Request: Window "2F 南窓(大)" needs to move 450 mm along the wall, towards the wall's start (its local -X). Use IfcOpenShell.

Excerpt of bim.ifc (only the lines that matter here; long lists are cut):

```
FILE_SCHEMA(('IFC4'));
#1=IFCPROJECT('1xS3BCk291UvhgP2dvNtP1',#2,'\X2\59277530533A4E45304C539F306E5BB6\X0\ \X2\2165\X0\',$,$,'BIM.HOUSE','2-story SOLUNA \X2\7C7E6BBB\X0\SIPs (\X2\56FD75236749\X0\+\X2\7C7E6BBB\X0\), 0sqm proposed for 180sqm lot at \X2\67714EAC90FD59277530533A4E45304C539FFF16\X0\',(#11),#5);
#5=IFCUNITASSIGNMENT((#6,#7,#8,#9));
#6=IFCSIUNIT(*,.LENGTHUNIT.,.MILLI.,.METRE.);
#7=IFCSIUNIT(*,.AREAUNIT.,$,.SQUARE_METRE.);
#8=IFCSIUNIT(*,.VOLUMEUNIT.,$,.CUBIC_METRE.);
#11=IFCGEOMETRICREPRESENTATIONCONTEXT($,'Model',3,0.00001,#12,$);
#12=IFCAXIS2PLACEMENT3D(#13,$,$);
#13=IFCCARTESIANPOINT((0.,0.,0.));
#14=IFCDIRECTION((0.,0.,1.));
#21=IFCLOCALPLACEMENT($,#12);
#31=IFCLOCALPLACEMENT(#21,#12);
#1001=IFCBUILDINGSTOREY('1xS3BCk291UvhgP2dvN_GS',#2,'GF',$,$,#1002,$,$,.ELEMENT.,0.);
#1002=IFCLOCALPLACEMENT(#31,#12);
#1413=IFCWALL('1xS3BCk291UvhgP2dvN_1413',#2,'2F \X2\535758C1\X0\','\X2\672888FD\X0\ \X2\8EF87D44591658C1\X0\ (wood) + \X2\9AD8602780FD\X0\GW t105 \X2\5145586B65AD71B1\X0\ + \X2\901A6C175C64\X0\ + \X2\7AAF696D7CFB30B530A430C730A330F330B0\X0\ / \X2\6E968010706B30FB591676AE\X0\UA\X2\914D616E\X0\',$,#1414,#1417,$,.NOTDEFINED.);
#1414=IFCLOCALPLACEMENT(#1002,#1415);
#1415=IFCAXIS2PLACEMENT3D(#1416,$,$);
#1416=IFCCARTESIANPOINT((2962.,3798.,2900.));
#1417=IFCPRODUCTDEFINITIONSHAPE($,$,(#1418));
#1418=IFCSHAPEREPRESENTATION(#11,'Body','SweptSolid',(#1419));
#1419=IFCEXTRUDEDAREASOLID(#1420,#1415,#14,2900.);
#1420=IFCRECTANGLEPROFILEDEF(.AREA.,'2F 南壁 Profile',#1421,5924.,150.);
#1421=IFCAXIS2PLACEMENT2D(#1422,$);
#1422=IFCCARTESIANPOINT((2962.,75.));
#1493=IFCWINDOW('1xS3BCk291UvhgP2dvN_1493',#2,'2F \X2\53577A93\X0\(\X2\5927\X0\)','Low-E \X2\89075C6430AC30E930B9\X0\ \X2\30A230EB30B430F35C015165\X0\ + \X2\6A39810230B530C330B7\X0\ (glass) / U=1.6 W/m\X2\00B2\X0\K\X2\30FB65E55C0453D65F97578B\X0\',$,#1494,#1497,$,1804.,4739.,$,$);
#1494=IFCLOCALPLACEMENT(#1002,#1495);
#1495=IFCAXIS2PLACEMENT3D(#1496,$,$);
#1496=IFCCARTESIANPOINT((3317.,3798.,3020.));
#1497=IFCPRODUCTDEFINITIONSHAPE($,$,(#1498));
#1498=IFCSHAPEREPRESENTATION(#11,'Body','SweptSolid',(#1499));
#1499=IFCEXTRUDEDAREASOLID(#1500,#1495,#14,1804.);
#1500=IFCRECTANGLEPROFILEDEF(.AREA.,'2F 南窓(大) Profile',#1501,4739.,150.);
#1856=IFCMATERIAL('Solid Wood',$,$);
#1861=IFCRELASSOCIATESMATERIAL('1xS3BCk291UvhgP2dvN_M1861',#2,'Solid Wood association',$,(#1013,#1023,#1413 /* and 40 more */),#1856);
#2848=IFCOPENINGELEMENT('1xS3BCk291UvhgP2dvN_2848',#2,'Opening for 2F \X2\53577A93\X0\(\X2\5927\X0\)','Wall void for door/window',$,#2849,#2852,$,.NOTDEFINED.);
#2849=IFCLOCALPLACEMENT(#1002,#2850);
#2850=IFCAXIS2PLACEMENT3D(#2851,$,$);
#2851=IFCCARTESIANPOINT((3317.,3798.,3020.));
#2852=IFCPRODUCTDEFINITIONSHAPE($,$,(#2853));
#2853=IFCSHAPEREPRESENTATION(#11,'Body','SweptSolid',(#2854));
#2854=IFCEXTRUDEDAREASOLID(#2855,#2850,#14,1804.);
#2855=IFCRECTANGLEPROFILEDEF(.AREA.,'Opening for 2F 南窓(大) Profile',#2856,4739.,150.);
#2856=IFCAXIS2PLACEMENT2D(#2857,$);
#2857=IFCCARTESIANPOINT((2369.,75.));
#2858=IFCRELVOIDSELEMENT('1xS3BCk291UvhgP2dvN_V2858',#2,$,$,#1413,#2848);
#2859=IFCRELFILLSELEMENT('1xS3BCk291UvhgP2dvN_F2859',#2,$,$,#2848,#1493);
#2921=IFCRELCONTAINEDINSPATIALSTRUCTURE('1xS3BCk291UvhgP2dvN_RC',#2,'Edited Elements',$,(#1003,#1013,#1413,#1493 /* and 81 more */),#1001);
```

```python
import ifcopenshell
import ifcopenshell.api.geometry
import ifcopenshell.util.placement
import ifcopenshell.util.unit

model = ifcopenshell.open("bim.ifc")
unit_scale = ifcopenshell.util.unit.calculate_unit_scale(model)

window = model.by_id(1493)
opening = window.FillsVoids[0].RelatingOpeningElement
wall = opening.VoidsElements[0].RelatingBuildingElement

wall_matrix = ifcopenshell.util.placement.get_local_placement(wall.ObjectPlacement)
shift = wall_matrix[:3, 0] * -0.45 / unit_scale
before = ifcopenshell.util.placement.get_local_placement(window.ObjectPlacement)[:3, 3].copy()

# The window is not placed relative to its opening, so move both.
for product in (opening, window):
    matrix = ifcopenshell.util.placement.get_local_placement(product.ObjectPlacement)
    matrix[:3, 3] += shift
    ifcopenshell.api.geometry.edit_object_placement(model, product=product, matrix=matrix, is_si=False)

after = ifcopenshell.util.placement.get_local_placement(window.ObjectPlacement)[:3, 3]
print("window moved by", (after - before).round(3) + 0.0)

model.write("bim_v2.ifc")
```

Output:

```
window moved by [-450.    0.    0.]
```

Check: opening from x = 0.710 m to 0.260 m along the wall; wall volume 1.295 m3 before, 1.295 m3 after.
